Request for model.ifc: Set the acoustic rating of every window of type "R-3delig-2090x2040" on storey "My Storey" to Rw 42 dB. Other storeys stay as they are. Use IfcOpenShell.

First a look at what the model holds.

```python
import ifcopenshell
import ifcopenshell.util.element

model = ifcopenshell.open("model.ifc")
print(model.schema)
storey = next(s for s in model.by_type("IfcBuildingStorey") if s.Name == "My Storey")
windows = [e for e in ifcopenshell.util.element.get_decomposition(storey) if e.is_a("IfcWindow")]
seen = {}
for e in windows:
    element_type = ifcopenshell.util.element.get_type(e)
    key = (element_type.Name if element_type != e and element_type else None, ifcopenshell.util.element.get_pset(e, "Pset_WindowCommon", "AcousticRating"))
    seen[key] = seen.get(key, 0) + 1
for (name, value), count in sorted(seen.items(), key=str):
    print(count, "x", name, "|", value)
```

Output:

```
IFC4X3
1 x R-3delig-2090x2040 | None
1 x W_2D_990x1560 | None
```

```python
import ifcopenshell
import ifcopenshell.api.pset
import ifcopenshell.util.element

model = ifcopenshell.open("model.ifc")

storey = next(s for s in model.by_type("IfcBuildingStorey") if s.Name == "My Storey")
windows = [e for e in ifcopenshell.util.element.get_decomposition(storey) if e.is_a("IfcWindow")]

count = 0
for e in windows:
    element_type = ifcopenshell.util.element.get_type(e)
    if element_type in (None, e) or element_type.Name != "R-3delig-2090x2040":
        continue
    # add_pset returns the element's existing set when there is one.
    pset = ifcopenshell.api.pset.add_pset(model, product=e, name="Pset_WindowCommon")
    ifcopenshell.api.pset.edit_pset(model, pset=pset, properties={"AcousticRating": "Rw 42 dB"})
    count += 1

print(count, "windows updated")

model.write("model_v2.ifc")
```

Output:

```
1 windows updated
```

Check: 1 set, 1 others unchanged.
